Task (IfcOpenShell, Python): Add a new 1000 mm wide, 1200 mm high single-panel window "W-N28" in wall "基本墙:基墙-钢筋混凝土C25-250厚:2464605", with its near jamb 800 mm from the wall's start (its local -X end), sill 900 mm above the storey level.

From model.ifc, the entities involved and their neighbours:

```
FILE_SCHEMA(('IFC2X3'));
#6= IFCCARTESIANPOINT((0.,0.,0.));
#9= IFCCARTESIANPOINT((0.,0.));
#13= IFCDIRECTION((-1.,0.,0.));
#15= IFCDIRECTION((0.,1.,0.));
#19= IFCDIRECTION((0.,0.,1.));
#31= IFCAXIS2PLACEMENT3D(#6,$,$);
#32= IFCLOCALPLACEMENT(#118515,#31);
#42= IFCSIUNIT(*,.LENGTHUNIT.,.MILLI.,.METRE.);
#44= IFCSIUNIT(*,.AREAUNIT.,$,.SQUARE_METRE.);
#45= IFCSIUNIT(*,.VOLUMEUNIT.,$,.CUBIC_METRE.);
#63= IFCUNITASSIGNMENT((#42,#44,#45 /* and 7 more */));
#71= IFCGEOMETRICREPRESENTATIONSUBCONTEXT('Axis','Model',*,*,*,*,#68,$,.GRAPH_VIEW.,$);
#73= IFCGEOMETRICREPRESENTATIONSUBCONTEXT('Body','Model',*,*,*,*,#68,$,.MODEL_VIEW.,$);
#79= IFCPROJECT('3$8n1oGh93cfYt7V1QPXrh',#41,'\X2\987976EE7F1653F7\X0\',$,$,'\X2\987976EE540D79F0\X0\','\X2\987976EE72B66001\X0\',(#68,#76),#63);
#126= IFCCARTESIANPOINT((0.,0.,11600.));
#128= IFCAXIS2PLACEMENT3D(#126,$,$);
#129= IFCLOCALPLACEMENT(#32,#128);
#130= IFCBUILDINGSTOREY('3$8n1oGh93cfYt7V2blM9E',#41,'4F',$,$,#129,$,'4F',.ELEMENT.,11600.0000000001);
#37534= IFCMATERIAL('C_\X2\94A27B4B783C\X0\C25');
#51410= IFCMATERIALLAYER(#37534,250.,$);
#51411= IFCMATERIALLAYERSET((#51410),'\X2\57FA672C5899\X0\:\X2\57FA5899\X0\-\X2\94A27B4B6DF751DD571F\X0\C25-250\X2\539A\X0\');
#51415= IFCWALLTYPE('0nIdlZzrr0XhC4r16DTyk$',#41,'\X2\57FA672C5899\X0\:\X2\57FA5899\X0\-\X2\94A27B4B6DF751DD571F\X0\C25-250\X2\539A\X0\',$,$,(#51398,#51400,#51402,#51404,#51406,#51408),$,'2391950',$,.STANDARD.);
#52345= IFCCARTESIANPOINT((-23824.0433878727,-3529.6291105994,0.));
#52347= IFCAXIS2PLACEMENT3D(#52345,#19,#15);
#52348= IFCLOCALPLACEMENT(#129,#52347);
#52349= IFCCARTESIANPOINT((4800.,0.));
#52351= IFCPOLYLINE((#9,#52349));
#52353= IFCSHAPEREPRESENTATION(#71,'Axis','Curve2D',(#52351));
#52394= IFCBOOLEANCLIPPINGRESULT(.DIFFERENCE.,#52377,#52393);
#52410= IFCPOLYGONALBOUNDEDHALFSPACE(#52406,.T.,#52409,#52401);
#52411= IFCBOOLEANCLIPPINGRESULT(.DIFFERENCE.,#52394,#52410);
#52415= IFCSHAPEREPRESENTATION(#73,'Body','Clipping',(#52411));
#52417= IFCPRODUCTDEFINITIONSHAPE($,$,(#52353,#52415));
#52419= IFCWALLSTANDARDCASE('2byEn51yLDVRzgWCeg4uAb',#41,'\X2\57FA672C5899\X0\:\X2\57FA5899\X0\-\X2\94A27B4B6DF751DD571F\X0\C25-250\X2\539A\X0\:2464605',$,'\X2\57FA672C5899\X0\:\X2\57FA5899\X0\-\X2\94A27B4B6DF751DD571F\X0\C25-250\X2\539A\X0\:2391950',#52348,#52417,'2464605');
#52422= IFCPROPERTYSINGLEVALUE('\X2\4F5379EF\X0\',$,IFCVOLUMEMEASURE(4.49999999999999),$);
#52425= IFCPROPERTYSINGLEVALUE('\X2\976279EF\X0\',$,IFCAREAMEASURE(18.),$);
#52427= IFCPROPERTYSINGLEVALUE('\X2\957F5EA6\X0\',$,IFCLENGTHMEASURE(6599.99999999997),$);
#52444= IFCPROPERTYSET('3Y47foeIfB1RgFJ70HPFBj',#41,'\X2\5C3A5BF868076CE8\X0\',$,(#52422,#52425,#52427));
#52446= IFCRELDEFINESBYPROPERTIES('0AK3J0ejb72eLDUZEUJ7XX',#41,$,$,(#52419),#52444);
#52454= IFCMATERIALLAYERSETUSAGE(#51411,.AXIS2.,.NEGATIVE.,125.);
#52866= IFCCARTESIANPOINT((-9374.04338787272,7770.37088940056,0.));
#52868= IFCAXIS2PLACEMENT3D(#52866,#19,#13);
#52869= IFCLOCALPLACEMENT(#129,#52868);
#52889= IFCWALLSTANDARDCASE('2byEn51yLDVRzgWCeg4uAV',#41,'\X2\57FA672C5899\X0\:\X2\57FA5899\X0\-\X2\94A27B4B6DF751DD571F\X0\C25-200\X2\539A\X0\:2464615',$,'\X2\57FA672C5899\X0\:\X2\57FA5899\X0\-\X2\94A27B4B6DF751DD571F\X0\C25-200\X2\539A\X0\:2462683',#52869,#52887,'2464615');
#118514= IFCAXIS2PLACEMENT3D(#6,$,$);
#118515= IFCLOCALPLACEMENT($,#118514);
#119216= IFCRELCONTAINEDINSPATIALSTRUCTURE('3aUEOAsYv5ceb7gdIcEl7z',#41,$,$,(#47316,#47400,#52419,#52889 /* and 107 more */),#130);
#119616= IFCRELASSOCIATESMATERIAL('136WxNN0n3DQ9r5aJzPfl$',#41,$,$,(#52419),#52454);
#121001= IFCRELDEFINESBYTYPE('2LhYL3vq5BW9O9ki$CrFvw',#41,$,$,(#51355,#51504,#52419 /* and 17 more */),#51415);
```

```python
import numpy as np
import ifcopenshell
import ifcopenshell.api.feature
import ifcopenshell.api.geometry
import ifcopenshell.api.pset
import ifcopenshell.api.root
import ifcopenshell.api.spatial
import ifcopenshell.api.type
import ifcopenshell.geom
import ifcopenshell.util.element
import ifcopenshell.util.placement
import ifcopenshell.util.representation
import ifcopenshell.util.shape
import ifcopenshell.util.unit

model = ifcopenshell.open("model.ifc")
unit_scale = ifcopenshell.util.unit.calculate_unit_scale(model)
area_scale = ifcopenshell.util.unit.calculate_unit_scale(model, "AREAUNIT")
volume_scale = ifcopenshell.util.unit.calculate_unit_scale(model, "VOLUMEUNIT")
settings = ifcopenshell.geom.settings()


def volume(element):
    """Net volume in cubic metres, openings subtracted."""
    shape = ifcopenshell.geom.create_shape(settings, element)
    return ifcopenshell.util.shape.get_volume(shape.geometry)


wall = model.by_guid("2byEn51yLDVRzgWCeg4uAb")
storey = ifcopenshell.util.element.get_container(wall, ifc_class="IfcBuildingStorey")
context = ifcopenshell.util.representation.get_context(model, "Model", "Body", "MODEL_VIEW")
before = volume(wall)

width, height, from_end, sill = 1, 1.2, 0.8, 0.9  # metres

# The wall runs along its own X axis, and the end named is its -X end.
wall_shape = ifcopenshell.geom.create_shape(settings, wall)
x, y, z = ifcopenshell.util.shape.get_vertices(wall_shape.geometry).T
start = x.min() + from_end
face, thickness = float(y.min()), float(y.max() - y.min())
wall_matrix = ifcopenshell.util.placement.get_local_placement(wall.ObjectPlacement)
level = ifcopenshell.util.placement.get_local_placement(storey.ObjectPlacement)[2, 3]


def in_wall(x, y):
    """Placement at x, y metres in the wall's axes, at sill height."""
    matrix = wall_matrix.copy()
    matrix[:, 3] = wall_matrix @ np.array([x / unit_scale, y / unit_scale, 0.0, 1.0])
    matrix[2, 3] = level + sill / unit_scale
    return matrix


# Opening: a box that overshoots both wall faces by 50 mm.
opening = ifcopenshell.api.root.create_entity(model, ifc_class="IfcOpeningElement")
box = ifcopenshell.api.geometry.add_wall_representation(
    model, context=context, length=width, height=height, thickness=thickness + 0.1
)
ifcopenshell.api.geometry.assign_representation(model, product=opening, representation=box)
ifcopenshell.api.geometry.edit_object_placement(model, product=opening, matrix=in_wall(start, face - 0.05), is_si=False)
ifcopenshell.api.feature.add_feature(model, feature=opening, element=wall)

window = ifcopenshell.api.root.create_entity(model, ifc_class="IfcWindow", name="W-N28")
window.OverallWidth, window.OverallHeight = width / unit_scale, height / unit_scale
body = ifcopenshell.api.geometry.add_window_representation(
    model,
    context=context,
    overall_width=window.OverallWidth,
    overall_height=window.OverallHeight,
    partition_type="SINGLE_PANEL",
)
ifcopenshell.api.geometry.assign_representation(model, product=window, representation=body)
ifcopenshell.api.spatial.assign_container(model, products=[window], relating_structure=storey)
fills = ifcopenshell.api.feature.add_filling(model, opening=opening, element=window)
fills.OwnerHistory = window.OwnerHistory  # required in IFC2X3

# IFC2X3 keeps the operation on the window style.
style = ifcopenshell.api.root.create_entity(model, ifc_class="IfcWindowStyle", name="W-N28")
style.OperationType, style.ConstructionType = "SINGLE_PANEL", "NOTDEFINED"
style.ParameterTakesPrecedence = style.Sizeable = False
ifcopenshell.api.type.assign_type(model, related_objects=[window], relating_type=style)

# Centre the window in the wall's thickness.
ifcopenshell.api.geometry.edit_object_placement(model, product=window, matrix=in_wall(start, face), is_si=False)
window_shape = ifcopenshell.geom.create_shape(settings, window)
depth = ifcopenshell.util.shape.get_vertices(window_shape.geometry)[:, 1]
offset = face + thickness / 2 - (depth.min() + depth.max()) / 2
ifcopenshell.api.geometry.edit_object_placement(model, product=window, matrix=in_wall(start, offset), is_si=False)

after = volume(wall)

# Update the wall's stored quantities.
pset = model.by_id(ifcopenshell.util.element.get_pset(wall, "尺寸标注", should_inherit=False)["id"])
ifcopenshell.api.pset.edit_pset(model, pset=pset, properties={
    "体积": model.create_entity("IfcVolumeMeasure", after / volume_scale),
    "面积": model.create_entity("IfcAreaMeasure", after / thickness / area_scale),
})

print(f"wall volume {before:.3f} -> {after:.3f} m3")

model.write("model-out.ifc")
```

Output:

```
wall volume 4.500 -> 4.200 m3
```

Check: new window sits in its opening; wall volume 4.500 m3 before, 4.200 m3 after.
